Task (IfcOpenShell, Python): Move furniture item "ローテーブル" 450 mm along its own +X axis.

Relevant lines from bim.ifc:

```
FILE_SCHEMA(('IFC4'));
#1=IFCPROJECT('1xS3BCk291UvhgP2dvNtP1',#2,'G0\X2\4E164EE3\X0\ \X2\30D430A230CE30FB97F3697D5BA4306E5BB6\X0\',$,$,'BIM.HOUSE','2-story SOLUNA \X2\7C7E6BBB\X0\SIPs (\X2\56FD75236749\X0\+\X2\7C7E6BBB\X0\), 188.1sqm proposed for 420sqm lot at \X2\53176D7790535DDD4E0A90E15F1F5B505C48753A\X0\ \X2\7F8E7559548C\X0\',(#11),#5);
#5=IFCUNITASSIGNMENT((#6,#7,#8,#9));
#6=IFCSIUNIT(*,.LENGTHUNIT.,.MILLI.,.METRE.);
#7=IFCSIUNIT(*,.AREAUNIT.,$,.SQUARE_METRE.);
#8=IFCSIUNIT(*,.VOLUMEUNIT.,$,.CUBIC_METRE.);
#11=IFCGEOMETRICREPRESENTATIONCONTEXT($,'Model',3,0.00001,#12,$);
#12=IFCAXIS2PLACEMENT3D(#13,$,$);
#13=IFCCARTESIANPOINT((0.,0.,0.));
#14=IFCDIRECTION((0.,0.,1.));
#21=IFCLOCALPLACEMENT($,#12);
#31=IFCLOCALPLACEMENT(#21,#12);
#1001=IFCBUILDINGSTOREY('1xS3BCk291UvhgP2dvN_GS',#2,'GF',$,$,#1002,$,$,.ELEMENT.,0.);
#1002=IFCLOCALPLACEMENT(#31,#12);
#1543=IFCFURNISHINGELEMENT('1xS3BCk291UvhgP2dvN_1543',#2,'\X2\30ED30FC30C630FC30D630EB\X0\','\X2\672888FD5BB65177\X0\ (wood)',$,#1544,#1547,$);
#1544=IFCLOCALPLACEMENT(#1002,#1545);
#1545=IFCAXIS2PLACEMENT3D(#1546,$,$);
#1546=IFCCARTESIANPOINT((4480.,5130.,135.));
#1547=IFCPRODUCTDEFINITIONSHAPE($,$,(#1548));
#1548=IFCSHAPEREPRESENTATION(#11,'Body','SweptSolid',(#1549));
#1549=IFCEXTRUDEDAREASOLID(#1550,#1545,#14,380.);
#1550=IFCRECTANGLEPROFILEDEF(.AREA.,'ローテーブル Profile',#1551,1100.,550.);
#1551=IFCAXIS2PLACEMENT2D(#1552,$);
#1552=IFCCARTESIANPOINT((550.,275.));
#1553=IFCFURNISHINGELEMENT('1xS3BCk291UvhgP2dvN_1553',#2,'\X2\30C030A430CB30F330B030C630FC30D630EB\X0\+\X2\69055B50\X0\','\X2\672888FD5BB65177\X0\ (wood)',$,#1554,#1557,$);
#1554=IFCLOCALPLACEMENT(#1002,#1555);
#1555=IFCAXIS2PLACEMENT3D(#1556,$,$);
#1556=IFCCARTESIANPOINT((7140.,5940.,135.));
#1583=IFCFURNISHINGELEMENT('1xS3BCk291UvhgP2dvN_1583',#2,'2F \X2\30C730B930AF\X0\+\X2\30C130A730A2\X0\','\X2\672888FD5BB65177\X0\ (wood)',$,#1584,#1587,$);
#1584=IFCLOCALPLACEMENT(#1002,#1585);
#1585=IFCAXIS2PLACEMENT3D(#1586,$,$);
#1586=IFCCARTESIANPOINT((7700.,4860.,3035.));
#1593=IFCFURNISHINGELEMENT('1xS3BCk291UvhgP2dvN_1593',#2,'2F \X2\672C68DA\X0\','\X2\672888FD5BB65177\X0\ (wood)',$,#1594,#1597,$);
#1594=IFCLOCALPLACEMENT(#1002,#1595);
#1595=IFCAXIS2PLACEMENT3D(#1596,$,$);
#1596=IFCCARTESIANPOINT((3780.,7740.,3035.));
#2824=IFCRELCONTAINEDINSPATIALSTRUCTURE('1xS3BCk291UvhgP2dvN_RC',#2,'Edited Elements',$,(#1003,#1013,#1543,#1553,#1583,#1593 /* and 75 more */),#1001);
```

```python
import ifcopenshell
import ifcopenshell.api.geometry
import ifcopenshell.util.placement

model = ifcopenshell.open("bim.ifc")

item = model.by_guid("1xS3BCk291UvhgP2dvN_1543")
matrix = ifcopenshell.util.placement.get_local_placement(item.ObjectPlacement)
matrix[:3, 3] += matrix[:3, 0] * 450.0
ifcopenshell.api.geometry.edit_object_placement(model, product=item, matrix=matrix, is_si=False)

print(ifcopenshell.util.placement.get_local_placement(item.ObjectPlacement).round(3) + 0.0)

model.write("bim_rev.ifc")
```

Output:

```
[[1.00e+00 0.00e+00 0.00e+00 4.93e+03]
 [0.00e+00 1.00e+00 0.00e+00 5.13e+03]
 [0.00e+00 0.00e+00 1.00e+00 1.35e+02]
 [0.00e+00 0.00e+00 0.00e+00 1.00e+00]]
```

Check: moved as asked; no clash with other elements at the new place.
